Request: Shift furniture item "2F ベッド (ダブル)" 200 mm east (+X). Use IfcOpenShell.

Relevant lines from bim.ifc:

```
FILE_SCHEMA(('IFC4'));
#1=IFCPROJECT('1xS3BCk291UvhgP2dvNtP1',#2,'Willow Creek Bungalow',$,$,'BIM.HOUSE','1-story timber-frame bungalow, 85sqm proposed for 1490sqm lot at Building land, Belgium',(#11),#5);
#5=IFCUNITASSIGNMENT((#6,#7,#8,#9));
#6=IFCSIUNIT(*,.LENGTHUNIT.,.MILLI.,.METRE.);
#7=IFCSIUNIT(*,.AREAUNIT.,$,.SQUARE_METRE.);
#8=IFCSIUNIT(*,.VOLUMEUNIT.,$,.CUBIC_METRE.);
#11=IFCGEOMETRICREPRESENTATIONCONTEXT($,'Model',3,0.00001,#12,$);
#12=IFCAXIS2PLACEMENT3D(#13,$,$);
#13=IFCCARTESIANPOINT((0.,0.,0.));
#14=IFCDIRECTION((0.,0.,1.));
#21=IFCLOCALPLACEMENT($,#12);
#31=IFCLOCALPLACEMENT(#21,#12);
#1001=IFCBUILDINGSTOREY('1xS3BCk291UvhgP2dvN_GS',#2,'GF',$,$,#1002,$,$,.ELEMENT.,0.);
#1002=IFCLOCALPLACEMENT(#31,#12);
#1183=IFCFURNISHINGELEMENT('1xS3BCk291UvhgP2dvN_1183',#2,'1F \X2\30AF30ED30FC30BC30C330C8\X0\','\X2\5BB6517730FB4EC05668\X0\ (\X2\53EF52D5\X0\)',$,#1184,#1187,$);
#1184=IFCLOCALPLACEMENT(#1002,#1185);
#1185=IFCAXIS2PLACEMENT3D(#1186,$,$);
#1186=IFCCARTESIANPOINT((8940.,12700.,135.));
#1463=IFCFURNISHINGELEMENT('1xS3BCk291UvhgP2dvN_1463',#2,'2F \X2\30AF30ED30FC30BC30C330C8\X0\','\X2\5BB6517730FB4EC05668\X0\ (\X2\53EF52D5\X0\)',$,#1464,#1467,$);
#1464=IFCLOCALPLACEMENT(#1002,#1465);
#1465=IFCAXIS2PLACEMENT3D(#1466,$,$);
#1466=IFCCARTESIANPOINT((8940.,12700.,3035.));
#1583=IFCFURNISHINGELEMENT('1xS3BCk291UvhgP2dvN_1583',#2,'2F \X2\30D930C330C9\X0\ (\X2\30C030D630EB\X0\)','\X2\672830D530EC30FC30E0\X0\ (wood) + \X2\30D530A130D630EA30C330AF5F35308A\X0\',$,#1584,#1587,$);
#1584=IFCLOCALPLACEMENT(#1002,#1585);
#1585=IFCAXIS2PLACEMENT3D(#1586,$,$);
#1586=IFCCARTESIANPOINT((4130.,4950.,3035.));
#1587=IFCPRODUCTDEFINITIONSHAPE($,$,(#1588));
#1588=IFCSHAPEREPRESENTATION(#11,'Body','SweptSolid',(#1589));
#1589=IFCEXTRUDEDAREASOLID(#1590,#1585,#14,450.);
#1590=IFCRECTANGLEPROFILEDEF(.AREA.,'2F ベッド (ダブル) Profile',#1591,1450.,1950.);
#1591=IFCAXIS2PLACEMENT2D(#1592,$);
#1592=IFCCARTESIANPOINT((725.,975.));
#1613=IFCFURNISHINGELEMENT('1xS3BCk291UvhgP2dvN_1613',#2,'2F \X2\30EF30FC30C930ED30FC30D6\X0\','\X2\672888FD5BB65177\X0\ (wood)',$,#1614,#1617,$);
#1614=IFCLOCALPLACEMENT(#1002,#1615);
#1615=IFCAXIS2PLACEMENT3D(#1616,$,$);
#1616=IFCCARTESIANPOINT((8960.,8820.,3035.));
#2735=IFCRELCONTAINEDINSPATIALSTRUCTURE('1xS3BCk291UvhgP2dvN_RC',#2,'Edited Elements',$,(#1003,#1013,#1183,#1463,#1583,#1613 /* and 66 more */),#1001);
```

```python
import ifcopenshell
import ifcopenshell.api.geometry
import ifcopenshell.util.placement

model = ifcopenshell.open("bim.ifc")

item = model.by_guid("1xS3BCk291UvhgP2dvN_1583")
matrix = ifcopenshell.util.placement.get_local_placement(item.ObjectPlacement)
matrix[0, 3] += 200.0
ifcopenshell.api.geometry.edit_object_placement(model, product=item, matrix=matrix, is_si=False)

print(ifcopenshell.util.placement.get_local_placement(item.ObjectPlacement).round(3) + 0.0)

model.write("bim-out.ifc")
```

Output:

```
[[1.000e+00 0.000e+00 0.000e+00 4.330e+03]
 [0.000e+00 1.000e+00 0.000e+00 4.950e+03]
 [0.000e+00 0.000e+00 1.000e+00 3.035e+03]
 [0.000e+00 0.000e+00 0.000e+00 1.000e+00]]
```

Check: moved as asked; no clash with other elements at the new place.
